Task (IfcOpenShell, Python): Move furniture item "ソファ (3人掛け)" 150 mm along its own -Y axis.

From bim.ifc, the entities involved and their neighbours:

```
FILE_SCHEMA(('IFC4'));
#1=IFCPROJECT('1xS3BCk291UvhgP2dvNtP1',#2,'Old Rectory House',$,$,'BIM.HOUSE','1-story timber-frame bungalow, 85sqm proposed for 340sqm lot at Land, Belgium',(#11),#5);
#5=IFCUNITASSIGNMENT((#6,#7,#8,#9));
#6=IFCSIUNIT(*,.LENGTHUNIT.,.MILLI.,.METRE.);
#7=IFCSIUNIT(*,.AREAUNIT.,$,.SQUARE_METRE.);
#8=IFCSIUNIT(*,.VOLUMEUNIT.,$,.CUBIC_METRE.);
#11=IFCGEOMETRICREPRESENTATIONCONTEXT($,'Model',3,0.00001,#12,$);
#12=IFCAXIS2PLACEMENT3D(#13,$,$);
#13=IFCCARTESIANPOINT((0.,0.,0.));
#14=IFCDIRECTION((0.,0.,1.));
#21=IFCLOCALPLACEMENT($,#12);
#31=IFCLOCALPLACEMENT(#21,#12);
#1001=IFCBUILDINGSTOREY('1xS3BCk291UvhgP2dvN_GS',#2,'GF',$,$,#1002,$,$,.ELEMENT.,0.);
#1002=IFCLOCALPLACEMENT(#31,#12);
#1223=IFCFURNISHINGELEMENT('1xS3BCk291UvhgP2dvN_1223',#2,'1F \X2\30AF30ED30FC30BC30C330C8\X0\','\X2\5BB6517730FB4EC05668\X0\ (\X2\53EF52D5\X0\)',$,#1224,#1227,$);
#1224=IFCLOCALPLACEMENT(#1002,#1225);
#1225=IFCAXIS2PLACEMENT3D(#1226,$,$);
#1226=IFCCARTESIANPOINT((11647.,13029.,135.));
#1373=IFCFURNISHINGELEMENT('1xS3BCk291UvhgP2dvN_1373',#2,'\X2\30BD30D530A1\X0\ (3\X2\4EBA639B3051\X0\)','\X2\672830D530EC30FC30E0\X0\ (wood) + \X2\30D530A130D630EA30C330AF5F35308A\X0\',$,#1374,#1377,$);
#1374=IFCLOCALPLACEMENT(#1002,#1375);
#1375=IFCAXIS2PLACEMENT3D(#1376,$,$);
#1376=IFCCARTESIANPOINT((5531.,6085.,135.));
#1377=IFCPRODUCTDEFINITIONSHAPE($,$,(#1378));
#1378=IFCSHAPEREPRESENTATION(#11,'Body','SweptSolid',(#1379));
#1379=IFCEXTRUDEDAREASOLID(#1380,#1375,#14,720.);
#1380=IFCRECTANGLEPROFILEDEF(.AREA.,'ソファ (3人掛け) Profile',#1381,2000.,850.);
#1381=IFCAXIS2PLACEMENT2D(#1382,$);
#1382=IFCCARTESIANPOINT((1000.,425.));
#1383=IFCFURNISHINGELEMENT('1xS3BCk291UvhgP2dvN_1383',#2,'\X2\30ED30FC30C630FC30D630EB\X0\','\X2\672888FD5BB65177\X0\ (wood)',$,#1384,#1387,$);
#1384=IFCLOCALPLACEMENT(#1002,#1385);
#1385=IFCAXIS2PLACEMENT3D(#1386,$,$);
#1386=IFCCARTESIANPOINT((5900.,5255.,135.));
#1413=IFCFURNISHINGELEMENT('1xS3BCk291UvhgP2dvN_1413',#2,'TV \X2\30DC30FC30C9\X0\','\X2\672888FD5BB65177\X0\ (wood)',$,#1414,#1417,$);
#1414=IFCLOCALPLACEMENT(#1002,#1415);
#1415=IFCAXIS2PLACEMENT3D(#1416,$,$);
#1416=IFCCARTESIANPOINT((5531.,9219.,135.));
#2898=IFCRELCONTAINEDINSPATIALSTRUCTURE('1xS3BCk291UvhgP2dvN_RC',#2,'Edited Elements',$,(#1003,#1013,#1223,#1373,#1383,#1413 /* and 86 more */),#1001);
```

```python
import ifcopenshell
import ifcopenshell.api.geometry
import ifcopenshell.util.placement
import ifcopenshell.util.unit

model = ifcopenshell.open("bim.ifc")
unit_scale = ifcopenshell.util.unit.calculate_unit_scale(model)

item = model.by_guid("1xS3BCk291UvhgP2dvN_1373")
matrix = ifcopenshell.util.placement.get_local_placement(item.ObjectPlacement)
matrix[:3, 3] -= matrix[:3, 1] * 0.15 / unit_scale
ifcopenshell.api.geometry.edit_object_placement(model, product=item, matrix=matrix, is_si=False)

print(ifcopenshell.util.placement.get_local_placement(item.ObjectPlacement).round(3) + 0.0)

model.write("bim_edited.ifc")
```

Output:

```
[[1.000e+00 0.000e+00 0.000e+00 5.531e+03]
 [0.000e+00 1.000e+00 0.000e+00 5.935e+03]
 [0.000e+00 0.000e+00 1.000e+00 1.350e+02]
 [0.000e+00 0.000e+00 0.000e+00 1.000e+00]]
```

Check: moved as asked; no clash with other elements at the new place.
